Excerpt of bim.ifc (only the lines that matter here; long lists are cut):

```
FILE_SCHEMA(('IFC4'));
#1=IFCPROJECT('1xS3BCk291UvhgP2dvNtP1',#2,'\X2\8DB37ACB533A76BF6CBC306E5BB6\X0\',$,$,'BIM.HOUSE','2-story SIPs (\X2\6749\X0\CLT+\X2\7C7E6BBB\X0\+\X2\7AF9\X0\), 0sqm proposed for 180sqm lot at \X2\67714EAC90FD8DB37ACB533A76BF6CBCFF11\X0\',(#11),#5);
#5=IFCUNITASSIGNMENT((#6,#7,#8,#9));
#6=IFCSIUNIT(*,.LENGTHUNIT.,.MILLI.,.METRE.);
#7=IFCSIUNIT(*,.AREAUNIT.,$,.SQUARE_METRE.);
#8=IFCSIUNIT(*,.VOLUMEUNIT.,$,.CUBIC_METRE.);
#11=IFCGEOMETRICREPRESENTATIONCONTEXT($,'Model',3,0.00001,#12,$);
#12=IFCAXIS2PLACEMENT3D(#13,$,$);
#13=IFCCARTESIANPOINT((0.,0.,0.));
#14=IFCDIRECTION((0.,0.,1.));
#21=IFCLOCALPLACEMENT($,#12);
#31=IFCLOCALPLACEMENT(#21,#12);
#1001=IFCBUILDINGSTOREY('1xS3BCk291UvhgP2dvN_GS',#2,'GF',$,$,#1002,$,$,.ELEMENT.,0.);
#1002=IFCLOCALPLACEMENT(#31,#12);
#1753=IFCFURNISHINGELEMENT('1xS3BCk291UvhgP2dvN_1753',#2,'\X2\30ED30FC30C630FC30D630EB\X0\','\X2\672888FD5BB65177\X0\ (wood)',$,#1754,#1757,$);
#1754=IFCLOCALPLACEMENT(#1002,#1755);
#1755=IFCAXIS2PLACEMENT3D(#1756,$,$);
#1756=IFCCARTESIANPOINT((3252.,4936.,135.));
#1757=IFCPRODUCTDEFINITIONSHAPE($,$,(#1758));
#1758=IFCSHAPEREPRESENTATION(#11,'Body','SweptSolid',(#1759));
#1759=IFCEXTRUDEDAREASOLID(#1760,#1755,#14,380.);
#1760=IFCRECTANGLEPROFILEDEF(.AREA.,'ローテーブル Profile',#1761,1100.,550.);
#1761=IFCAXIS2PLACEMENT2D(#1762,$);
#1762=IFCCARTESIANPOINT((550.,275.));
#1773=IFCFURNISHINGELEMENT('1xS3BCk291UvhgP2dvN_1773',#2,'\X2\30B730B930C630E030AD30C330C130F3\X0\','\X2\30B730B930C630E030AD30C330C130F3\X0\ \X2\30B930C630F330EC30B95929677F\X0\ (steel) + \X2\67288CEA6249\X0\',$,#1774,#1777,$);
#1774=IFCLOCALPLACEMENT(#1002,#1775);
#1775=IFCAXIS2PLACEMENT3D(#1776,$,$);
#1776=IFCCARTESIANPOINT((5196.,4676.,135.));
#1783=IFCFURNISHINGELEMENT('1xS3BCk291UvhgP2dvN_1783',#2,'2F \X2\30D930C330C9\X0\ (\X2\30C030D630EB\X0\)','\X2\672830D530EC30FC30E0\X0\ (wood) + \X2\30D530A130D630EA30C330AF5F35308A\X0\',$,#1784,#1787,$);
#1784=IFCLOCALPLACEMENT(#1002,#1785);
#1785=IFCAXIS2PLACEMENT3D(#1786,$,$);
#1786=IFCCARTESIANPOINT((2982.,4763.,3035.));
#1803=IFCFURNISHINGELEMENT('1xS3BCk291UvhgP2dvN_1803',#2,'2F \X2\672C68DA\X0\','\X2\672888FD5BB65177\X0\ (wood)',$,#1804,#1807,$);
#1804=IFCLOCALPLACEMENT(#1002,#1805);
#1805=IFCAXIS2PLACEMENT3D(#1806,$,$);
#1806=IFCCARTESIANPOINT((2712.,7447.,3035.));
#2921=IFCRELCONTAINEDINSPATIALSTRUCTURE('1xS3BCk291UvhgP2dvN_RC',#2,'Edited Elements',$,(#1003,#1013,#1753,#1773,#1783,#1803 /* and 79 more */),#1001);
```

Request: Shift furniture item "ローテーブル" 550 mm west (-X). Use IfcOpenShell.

```python
import ifcopenshell
import ifcopenshell.api.geometry
import ifcopenshell.util.placement

model = ifcopenshell.open("bim.ifc")

item = model.by_guid("1xS3BCk291UvhgP2dvN_1753")
matrix = ifcopenshell.util.placement.get_local_placement(item.ObjectPlacement)
matrix[0, 3] -= 550.0
ifcopenshell.api.geometry.edit_object_placement(model, product=item, matrix=matrix, is_si=False)

print(ifcopenshell.util.placement.get_local_placement(item.ObjectPlacement).round(3) + 0.0)

model.write("bim_rev.ifc")
```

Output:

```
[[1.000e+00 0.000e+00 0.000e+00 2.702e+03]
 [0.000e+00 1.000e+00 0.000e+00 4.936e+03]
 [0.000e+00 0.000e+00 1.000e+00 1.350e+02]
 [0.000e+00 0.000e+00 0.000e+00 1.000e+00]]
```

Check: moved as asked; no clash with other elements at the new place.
